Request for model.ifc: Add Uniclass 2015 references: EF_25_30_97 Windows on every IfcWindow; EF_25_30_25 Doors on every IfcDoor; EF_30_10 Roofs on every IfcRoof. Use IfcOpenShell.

First a look at what the model holds.

```python
import ifcopenshell

model = ifcopenshell.open("model.ifc")
print(model.schema)
print("classifications:", [c.Name for c in model.by_type("IfcClassification")])
for ifc_class in ("IfcDoor", "IfcRoof", "IfcStair", "IfcWall", "IfcWindow"):
    print(ifc_class, len(model.by_type(ifc_class)))
```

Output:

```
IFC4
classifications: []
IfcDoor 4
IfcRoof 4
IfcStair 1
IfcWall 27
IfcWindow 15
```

```python
import ifcopenshell
import ifcopenshell.api.classification

model = ifcopenshell.open("model.ifc")

system = ifcopenshell.api.classification.add_classification(model, classification="Uniclass 2015")

codes = {
    "IfcWindow": ("EF_25_30_97", "Windows"),
    "IfcDoor": ("EF_25_30_25", "Doors"),
    "IfcRoof": ("EF_30_10", "Roofs"),
}
for ifc_class, (code, name) in codes.items():
    products = model.by_type(ifc_class)
    ifcopenshell.api.classification.add_reference(
        model, products=products, classification=system, identification=code, name=name
    )
    print(code, len(products))

model.write("model_rev.ifc")
```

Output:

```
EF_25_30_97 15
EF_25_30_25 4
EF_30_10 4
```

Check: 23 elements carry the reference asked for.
